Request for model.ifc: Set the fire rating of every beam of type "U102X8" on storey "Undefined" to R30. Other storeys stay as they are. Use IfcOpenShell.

First a look at what the model holds.

```python
import ifcopenshell
import ifcopenshell.util.element

model = ifcopenshell.open("model.ifc")
print(model.schema)
storey = next(s for s in model.by_type("IfcBuildingStorey") if s.Name == "Undefined")
beams = [e for e in ifcopenshell.util.element.get_decomposition(storey) if e.is_a("IfcBeam")]
seen = {}
for e in beams:
    element_type = ifcopenshell.util.element.get_type(e)
    key = (element_type.Name if element_type != e and element_type else None, ifcopenshell.util.element.get_pset(e, "Pset_BeamCommon", "FireRating"))
    seen[key] = seen.get(key, 0) + 1
for (name, value), count in sorted(seen.items(), key=str):
    print(count, "x", name, "|", value)
```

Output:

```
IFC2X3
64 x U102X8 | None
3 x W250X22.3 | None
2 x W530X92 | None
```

```python
import ifcopenshell
import ifcopenshell.api.pset
import ifcopenshell.util.element

model = ifcopenshell.open("model.ifc")

storey = next(s for s in model.by_type("IfcBuildingStorey") if s.Name == "Undefined")
beams = [e for e in ifcopenshell.util.element.get_decomposition(storey) if e.is_a("IfcBeam")]

count = 0
for e in beams:
    element_type = ifcopenshell.util.element.get_type(e)
    if element_type in (None, e) or element_type.Name != "U102X8":
        continue
    found = ifcopenshell.util.element.get_pset(e, "Pset_BeamCommon", should_inherit=False)
    if found:
        pset = model.by_id(found["id"])
        if len(ifcopenshell.util.element.get_elements_by_pset(pset)) > 1:
            pset = ifcopenshell.api.pset.unshare_pset(model, products=[e], pset=pset)[0]
    else:
        pset = ifcopenshell.api.pset.add_pset(model, product=e, name="Pset_BeamCommon")
    ifcopenshell.api.pset.edit_pset(model, pset=pset, properties={"FireRating": "R30"})
    count += 1

print(count, "beams updated")

model.write("model_edited.ifc")
```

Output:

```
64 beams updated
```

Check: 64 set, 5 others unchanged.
